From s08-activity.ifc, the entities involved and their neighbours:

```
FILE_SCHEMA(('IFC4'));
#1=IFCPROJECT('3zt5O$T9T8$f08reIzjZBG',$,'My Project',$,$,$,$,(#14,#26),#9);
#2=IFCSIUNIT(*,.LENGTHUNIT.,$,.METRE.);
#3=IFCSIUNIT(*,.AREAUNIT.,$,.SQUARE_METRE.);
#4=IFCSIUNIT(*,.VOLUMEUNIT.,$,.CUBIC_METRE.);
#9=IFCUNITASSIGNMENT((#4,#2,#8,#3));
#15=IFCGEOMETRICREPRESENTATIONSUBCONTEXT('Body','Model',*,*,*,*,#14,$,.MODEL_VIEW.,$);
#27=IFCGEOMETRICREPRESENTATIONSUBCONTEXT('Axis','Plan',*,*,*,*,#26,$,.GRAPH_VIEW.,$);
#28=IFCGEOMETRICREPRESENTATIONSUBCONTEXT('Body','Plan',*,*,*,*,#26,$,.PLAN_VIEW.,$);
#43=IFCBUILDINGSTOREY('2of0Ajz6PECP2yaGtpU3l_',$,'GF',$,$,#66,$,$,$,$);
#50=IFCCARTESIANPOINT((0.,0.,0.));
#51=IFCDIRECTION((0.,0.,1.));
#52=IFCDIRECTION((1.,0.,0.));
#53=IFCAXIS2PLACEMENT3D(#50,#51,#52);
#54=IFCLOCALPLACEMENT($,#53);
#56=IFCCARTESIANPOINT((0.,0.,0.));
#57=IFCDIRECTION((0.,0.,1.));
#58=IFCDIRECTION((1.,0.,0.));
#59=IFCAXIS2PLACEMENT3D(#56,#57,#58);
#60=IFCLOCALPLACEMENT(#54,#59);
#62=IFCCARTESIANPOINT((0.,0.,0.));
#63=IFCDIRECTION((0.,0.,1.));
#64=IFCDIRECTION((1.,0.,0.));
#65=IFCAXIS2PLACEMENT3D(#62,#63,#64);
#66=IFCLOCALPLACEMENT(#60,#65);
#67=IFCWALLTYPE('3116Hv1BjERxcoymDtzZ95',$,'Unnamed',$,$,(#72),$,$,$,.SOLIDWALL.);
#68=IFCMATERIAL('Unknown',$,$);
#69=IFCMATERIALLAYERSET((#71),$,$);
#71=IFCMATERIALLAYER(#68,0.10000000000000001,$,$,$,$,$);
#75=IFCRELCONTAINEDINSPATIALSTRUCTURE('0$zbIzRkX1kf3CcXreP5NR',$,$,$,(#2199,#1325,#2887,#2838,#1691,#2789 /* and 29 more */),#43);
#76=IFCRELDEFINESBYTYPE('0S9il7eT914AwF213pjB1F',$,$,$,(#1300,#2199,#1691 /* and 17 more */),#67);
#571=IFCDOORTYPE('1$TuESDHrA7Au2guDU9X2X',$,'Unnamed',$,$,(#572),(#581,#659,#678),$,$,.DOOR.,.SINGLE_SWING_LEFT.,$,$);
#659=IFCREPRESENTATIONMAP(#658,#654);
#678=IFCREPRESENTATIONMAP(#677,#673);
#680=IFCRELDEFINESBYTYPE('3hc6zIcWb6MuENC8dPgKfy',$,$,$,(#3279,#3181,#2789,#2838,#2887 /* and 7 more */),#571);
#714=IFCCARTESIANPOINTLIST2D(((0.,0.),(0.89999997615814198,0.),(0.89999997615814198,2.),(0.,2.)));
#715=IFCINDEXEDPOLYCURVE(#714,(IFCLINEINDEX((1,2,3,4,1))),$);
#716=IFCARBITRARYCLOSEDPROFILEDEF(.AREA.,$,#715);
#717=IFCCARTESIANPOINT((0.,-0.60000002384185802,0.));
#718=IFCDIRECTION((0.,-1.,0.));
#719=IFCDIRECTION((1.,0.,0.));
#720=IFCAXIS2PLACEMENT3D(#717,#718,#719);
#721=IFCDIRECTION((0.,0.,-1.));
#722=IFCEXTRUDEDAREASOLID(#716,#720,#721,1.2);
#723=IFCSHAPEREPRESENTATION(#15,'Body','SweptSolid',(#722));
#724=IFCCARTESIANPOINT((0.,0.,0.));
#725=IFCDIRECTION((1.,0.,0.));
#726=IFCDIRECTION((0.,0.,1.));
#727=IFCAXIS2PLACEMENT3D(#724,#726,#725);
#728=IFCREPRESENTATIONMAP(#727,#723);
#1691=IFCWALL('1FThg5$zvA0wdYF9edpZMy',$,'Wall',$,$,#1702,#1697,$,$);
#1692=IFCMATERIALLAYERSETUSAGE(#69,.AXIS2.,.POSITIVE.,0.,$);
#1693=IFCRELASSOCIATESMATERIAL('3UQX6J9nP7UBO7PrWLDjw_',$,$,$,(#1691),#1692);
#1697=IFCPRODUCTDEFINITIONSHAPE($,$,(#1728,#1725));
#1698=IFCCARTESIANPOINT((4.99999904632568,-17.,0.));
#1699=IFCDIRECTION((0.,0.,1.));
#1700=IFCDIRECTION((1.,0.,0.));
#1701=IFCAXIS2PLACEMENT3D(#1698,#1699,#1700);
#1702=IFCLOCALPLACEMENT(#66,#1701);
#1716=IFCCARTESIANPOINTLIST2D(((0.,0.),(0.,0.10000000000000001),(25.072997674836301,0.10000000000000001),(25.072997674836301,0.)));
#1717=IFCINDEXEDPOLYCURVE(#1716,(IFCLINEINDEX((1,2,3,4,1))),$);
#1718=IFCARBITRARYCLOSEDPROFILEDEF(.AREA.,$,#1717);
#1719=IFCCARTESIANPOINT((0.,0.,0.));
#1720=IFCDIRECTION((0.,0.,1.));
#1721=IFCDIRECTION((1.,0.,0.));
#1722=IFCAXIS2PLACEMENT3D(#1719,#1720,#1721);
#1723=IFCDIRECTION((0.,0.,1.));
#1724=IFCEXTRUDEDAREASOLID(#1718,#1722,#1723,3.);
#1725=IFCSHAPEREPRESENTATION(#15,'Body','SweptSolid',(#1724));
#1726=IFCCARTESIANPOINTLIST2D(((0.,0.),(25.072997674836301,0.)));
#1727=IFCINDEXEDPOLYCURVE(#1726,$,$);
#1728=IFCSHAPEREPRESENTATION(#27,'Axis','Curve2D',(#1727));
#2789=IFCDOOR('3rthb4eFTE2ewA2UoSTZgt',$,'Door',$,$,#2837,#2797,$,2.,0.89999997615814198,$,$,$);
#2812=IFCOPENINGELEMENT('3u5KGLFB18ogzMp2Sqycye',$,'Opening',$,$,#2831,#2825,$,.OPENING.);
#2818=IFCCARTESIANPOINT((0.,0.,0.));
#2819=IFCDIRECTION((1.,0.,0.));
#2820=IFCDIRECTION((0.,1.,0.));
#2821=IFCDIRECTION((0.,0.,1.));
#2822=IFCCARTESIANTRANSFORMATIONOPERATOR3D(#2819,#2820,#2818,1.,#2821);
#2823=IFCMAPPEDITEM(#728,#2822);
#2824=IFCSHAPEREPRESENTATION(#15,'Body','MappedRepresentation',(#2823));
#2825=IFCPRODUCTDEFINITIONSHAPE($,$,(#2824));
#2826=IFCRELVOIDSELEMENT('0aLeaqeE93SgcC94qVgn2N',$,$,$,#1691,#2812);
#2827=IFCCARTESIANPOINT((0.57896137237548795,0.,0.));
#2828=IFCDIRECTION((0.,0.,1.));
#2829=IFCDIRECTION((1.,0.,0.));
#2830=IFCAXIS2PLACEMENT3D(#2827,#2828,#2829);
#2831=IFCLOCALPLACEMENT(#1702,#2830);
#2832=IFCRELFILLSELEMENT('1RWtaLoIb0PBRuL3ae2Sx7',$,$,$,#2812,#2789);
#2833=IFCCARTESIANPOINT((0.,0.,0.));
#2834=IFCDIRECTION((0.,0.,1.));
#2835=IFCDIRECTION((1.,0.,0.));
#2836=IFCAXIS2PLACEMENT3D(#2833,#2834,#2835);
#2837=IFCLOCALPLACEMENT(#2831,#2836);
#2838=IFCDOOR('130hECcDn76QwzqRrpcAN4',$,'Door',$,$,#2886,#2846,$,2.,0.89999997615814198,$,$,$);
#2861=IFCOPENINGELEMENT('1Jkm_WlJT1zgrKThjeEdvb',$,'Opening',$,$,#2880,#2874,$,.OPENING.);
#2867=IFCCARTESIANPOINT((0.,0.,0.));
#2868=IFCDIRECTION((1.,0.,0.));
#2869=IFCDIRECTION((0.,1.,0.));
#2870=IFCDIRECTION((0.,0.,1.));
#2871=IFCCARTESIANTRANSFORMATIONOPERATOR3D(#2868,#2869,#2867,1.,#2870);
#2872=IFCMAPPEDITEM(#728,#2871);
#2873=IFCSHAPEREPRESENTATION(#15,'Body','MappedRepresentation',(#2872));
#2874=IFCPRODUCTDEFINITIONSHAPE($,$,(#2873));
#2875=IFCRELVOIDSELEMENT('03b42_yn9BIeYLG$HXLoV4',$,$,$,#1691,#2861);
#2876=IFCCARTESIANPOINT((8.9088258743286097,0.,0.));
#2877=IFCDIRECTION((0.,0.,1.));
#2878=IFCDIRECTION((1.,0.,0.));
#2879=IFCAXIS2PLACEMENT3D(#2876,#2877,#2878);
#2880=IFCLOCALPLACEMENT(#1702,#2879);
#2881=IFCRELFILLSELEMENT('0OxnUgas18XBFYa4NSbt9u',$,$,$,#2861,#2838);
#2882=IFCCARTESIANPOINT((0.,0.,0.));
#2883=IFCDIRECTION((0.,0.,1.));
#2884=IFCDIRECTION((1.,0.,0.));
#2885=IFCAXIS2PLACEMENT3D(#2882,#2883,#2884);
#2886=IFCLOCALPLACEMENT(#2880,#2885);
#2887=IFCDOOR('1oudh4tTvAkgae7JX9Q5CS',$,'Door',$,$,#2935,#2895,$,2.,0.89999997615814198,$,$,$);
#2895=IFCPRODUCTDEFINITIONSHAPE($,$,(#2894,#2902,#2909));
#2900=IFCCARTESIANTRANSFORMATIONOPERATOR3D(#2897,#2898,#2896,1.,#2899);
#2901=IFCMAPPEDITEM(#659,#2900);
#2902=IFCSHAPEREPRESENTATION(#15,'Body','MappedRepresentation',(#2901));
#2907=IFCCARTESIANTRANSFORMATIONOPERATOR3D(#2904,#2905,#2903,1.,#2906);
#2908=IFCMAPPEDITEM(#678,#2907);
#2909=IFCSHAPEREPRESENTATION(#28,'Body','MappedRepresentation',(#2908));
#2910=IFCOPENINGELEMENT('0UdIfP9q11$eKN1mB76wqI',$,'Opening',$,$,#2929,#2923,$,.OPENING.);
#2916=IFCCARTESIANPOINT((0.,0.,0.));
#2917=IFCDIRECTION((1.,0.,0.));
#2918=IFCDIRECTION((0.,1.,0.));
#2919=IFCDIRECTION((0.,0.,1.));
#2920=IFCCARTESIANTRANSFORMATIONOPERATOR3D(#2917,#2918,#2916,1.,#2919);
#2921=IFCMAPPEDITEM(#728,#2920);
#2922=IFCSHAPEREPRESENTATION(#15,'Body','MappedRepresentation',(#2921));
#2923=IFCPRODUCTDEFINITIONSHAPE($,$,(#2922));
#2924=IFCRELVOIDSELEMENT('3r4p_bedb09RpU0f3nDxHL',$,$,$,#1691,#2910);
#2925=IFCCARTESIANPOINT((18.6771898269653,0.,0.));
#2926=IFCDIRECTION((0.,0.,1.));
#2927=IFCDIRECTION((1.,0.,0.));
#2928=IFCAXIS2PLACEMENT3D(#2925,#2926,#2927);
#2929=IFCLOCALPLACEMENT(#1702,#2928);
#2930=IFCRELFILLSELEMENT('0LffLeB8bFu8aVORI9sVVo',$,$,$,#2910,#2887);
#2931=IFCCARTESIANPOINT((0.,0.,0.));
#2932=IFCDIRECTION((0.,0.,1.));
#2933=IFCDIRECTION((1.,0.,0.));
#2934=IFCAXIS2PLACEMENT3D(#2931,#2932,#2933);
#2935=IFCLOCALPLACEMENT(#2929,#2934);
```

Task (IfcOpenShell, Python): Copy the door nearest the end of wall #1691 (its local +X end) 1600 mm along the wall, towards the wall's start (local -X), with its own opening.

```python
import ifcopenshell
import ifcopenshell.api.feature
import ifcopenshell.api.geometry
import ifcopenshell.api.root
import ifcopenshell.geom
import ifcopenshell.util.element
import ifcopenshell.util.placement
import ifcopenshell.util.shape
import ifcopenshell.util.unit

model = ifcopenshell.open("s08-activity.ifc")
unit_scale = ifcopenshell.util.unit.calculate_unit_scale(model)
settings = ifcopenshell.geom.settings()


def volume(element):
    """Net volume in cubic metres, openings subtracted."""
    shape = ifcopenshell.geom.create_shape(settings, element)
    return ifcopenshell.util.shape.get_volume(shape.geometry)


door = model.by_guid("1oudh4tTvAkgae7JX9Q5CS")
opening = door.FillsVoids[0].RelatingOpeningElement
wall = opening.VoidsElements[0].RelatingBuildingElement
before = volume(wall)
shift = ifcopenshell.util.placement.get_local_placement(wall.ObjectPlacement)[:3, 0] * -1.6 / unit_scale

# copy_class copies the void relationship, type, container and properties, but no geometry.
new_opening = ifcopenshell.api.root.copy_class(model, product=opening)
new_opening.Representation = ifcopenshell.util.element.copy_deep(
    model, opening.Representation, exclude=["IfcGeometricRepresentationContext", "IfcRepresentationMap"]
)
new_door = ifcopenshell.api.root.copy_class(model, product=door)
new_door.Representation = ifcopenshell.util.element.copy_deep(
    model, door.Representation, exclude=["IfcGeometricRepresentationContext", "IfcRepresentationMap"]
)
ifcopenshell.api.feature.add_filling(model, opening=new_opening, element=new_door)

for old, new in ((opening, new_opening), (door, new_door)):
    matrix = ifcopenshell.util.placement.get_local_placement(old.ObjectPlacement)
    matrix[:3, 3] += shift
    ifcopenshell.api.geometry.edit_object_placement(model, product=new, matrix=matrix, is_si=False)

after = volume(wall)

print(f"wall volume {before:.3f} -> {after:.3f} m3")

model.write("s08-activity_updated.ifc")
```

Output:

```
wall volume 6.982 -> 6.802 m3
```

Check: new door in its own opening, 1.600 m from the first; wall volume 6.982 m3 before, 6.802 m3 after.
